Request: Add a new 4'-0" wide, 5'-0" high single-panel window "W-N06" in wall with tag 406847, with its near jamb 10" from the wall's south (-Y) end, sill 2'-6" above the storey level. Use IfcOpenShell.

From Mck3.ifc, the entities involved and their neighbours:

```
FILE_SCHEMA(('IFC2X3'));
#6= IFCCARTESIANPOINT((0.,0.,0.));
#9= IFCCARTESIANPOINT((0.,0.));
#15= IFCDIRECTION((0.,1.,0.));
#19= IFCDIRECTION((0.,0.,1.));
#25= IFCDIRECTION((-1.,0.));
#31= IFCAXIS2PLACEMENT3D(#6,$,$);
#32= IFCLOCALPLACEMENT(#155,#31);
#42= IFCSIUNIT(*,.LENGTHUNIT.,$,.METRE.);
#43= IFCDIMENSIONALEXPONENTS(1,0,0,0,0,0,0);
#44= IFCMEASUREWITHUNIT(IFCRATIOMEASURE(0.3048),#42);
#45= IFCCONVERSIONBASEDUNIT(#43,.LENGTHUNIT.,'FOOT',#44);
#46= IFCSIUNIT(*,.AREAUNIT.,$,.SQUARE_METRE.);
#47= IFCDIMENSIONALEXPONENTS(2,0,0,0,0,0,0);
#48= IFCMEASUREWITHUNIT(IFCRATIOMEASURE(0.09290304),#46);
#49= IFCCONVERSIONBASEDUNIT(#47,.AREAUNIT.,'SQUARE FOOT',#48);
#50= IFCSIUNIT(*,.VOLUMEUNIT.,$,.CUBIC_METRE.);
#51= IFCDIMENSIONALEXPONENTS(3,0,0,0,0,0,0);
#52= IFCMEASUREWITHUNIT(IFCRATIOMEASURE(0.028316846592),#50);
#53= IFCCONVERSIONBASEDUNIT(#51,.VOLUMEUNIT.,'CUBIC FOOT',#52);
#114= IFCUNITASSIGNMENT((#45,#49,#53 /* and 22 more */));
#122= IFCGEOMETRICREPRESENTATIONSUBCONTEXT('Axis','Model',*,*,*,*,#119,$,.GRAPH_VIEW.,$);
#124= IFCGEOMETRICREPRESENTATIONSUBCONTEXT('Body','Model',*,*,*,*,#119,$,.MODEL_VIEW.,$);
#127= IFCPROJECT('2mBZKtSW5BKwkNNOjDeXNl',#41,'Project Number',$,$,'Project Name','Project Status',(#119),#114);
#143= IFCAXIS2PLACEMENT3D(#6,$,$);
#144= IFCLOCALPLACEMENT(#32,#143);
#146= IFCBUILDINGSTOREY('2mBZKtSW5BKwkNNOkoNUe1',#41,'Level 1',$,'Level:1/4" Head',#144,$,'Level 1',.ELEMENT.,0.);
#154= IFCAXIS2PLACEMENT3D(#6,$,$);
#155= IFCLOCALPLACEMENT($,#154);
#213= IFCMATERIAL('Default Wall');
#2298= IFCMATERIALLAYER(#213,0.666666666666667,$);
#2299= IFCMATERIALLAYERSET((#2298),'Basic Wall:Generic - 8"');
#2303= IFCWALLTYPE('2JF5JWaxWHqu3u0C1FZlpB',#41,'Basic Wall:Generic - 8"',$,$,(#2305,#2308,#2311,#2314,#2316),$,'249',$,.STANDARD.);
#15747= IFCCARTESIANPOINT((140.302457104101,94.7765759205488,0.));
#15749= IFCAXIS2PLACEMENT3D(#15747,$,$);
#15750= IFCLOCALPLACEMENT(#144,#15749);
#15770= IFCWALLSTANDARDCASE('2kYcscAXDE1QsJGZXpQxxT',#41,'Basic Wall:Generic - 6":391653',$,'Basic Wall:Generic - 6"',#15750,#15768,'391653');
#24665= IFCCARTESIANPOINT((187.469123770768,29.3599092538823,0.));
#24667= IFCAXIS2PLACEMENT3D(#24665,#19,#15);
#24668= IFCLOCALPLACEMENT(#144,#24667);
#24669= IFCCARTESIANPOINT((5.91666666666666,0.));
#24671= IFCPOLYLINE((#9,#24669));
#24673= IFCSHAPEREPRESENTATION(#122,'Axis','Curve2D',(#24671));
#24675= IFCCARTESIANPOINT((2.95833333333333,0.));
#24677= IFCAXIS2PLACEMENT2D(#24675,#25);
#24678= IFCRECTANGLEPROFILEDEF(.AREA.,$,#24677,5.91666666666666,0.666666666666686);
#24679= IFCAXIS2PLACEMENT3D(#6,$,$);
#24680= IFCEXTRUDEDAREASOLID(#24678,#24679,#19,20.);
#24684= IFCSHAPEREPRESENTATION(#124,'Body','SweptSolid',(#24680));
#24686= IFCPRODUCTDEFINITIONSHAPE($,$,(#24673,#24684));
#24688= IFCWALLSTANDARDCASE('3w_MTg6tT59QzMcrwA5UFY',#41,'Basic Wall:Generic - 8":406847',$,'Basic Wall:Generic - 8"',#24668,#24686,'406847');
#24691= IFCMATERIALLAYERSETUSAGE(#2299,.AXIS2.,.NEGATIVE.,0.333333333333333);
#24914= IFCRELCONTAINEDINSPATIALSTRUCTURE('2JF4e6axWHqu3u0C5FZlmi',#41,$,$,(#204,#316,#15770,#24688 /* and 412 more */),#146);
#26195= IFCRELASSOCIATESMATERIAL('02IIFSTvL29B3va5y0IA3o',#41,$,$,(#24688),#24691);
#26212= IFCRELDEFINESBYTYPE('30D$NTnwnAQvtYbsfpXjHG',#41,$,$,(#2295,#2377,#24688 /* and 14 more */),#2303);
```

```python
import numpy as np
import ifcopenshell
import ifcopenshell.api.feature
import ifcopenshell.api.geometry
import ifcopenshell.api.root
import ifcopenshell.api.spatial
import ifcopenshell.api.type
import ifcopenshell.geom
import ifcopenshell.util.element
import ifcopenshell.util.placement
import ifcopenshell.util.representation
import ifcopenshell.util.shape
import ifcopenshell.util.unit

model = ifcopenshell.open("Mck3.ifc")
unit_scale = ifcopenshell.util.unit.calculate_unit_scale(model)
settings = ifcopenshell.geom.settings()


def volume(element):
    """Net volume in cubic metres, openings subtracted."""
    shape = ifcopenshell.geom.create_shape(settings, element)
    return ifcopenshell.util.shape.get_volume(shape.geometry)


wall = model.by_id(24688)
storey = ifcopenshell.util.element.get_container(wall, ifc_class="IfcBuildingStorey")
context = ifcopenshell.util.representation.get_context(model, "Model", "Body", "MODEL_VIEW")
before = volume(wall)

width, height, from_end, sill = 1.2192, 1.524, 0.254, 0.762  # metres

# The wall runs along its own X axis, and the end named is its -X end.
wall_shape = ifcopenshell.geom.create_shape(settings, wall)
x, y, z = ifcopenshell.util.shape.get_vertices(wall_shape.geometry).T
start = x.min() + from_end
face, thickness = float(y.min()), float(y.max() - y.min())
wall_matrix = ifcopenshell.util.placement.get_local_placement(wall.ObjectPlacement)
level = ifcopenshell.util.placement.get_local_placement(storey.ObjectPlacement)[2, 3]


def in_wall(x, y):
    """Placement at x, y metres in the wall's axes, at sill height."""
    matrix = wall_matrix.copy()
    matrix[:, 3] = wall_matrix @ np.array([x / unit_scale, y / unit_scale, 0.0, 1.0])
    matrix[2, 3] = level + sill / unit_scale
    return matrix


# Opening: a box that overshoots both wall faces by 50 mm.
opening = ifcopenshell.api.root.create_entity(model, ifc_class="IfcOpeningElement")
box = ifcopenshell.api.geometry.add_wall_representation(
    model, context=context, length=width, height=height, thickness=thickness + 0.1
)
ifcopenshell.api.geometry.assign_representation(model, product=opening, representation=box)
ifcopenshell.api.geometry.edit_object_placement(model, product=opening, matrix=in_wall(start, face - 0.05), is_si=False)
ifcopenshell.api.feature.add_feature(model, feature=opening, element=wall)

window = ifcopenshell.api.root.create_entity(model, ifc_class="IfcWindow", name="W-N06")
window.OverallWidth, window.OverallHeight = width / unit_scale, height / unit_scale
body = ifcopenshell.api.geometry.add_window_representation(
    model,
    context=context,
    overall_width=window.OverallWidth,
    overall_height=window.OverallHeight,
    partition_type="SINGLE_PANEL",
)
ifcopenshell.api.geometry.assign_representation(model, product=window, representation=body)
ifcopenshell.api.spatial.assign_container(model, products=[window], relating_structure=storey)
fills = ifcopenshell.api.feature.add_filling(model, opening=opening, element=window)
fills.OwnerHistory = window.OwnerHistory  # required in IFC2X3

# IFC2X3 keeps the operation on the window style.
style = ifcopenshell.api.root.create_entity(model, ifc_class="IfcWindowStyle", name="W-N06")
style.OperationType, style.ConstructionType = "SINGLE_PANEL", "NOTDEFINED"
style.ParameterTakesPrecedence = style.Sizeable = False
ifcopenshell.api.type.assign_type(model, related_objects=[window], relating_type=style)

# Centre the window in the wall's thickness.
ifcopenshell.api.geometry.edit_object_placement(model, product=window, matrix=in_wall(start, face), is_si=False)
window_shape = ifcopenshell.geom.create_shape(settings, window)
depth = ifcopenshell.util.shape.get_vertices(window_shape.geometry)[:, 1]
offset = face + thickness / 2 - (depth.min() + depth.max()) / 2
ifcopenshell.api.geometry.edit_object_placement(model, product=window, matrix=in_wall(start, offset), is_si=False)

after = volume(wall)

print(f"wall volume {before:.3f} -> {after:.3f} m3")

model.write("Mck3_updated.ifc")
```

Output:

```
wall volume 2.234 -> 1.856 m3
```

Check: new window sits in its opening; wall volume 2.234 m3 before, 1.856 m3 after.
